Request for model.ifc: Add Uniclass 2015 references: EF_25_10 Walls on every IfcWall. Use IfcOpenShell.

First a look at what the model holds.

```python
import ifcopenshell

model = ifcopenshell.open("model.ifc")
print(model.schema)
print("classifications:", [c.Name for c in model.by_type("IfcClassification")])
for ifc_class in ("IfcDoor", "IfcRoof", "IfcStair", "IfcWall", "IfcWindow"):
    print(ifc_class, len(model.by_type(ifc_class)))
```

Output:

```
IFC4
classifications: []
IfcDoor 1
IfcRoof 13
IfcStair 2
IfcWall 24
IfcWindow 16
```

```python
import ifcopenshell
import ifcopenshell.api.classification

model = ifcopenshell.open("model.ifc")

system = ifcopenshell.api.classification.add_classification(model, classification="Uniclass 2015")

codes = {
    "IfcWall": ("EF_25_10", "Walls"),
}
for ifc_class, (code, name) in codes.items():
    products = model.by_type(ifc_class)
    ifcopenshell.api.classification.add_reference(
        model, products=products, classification=system, identification=code, name=name
    )
    print(code, len(products))

model.write("model_edited.ifc")
```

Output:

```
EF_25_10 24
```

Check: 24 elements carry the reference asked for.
